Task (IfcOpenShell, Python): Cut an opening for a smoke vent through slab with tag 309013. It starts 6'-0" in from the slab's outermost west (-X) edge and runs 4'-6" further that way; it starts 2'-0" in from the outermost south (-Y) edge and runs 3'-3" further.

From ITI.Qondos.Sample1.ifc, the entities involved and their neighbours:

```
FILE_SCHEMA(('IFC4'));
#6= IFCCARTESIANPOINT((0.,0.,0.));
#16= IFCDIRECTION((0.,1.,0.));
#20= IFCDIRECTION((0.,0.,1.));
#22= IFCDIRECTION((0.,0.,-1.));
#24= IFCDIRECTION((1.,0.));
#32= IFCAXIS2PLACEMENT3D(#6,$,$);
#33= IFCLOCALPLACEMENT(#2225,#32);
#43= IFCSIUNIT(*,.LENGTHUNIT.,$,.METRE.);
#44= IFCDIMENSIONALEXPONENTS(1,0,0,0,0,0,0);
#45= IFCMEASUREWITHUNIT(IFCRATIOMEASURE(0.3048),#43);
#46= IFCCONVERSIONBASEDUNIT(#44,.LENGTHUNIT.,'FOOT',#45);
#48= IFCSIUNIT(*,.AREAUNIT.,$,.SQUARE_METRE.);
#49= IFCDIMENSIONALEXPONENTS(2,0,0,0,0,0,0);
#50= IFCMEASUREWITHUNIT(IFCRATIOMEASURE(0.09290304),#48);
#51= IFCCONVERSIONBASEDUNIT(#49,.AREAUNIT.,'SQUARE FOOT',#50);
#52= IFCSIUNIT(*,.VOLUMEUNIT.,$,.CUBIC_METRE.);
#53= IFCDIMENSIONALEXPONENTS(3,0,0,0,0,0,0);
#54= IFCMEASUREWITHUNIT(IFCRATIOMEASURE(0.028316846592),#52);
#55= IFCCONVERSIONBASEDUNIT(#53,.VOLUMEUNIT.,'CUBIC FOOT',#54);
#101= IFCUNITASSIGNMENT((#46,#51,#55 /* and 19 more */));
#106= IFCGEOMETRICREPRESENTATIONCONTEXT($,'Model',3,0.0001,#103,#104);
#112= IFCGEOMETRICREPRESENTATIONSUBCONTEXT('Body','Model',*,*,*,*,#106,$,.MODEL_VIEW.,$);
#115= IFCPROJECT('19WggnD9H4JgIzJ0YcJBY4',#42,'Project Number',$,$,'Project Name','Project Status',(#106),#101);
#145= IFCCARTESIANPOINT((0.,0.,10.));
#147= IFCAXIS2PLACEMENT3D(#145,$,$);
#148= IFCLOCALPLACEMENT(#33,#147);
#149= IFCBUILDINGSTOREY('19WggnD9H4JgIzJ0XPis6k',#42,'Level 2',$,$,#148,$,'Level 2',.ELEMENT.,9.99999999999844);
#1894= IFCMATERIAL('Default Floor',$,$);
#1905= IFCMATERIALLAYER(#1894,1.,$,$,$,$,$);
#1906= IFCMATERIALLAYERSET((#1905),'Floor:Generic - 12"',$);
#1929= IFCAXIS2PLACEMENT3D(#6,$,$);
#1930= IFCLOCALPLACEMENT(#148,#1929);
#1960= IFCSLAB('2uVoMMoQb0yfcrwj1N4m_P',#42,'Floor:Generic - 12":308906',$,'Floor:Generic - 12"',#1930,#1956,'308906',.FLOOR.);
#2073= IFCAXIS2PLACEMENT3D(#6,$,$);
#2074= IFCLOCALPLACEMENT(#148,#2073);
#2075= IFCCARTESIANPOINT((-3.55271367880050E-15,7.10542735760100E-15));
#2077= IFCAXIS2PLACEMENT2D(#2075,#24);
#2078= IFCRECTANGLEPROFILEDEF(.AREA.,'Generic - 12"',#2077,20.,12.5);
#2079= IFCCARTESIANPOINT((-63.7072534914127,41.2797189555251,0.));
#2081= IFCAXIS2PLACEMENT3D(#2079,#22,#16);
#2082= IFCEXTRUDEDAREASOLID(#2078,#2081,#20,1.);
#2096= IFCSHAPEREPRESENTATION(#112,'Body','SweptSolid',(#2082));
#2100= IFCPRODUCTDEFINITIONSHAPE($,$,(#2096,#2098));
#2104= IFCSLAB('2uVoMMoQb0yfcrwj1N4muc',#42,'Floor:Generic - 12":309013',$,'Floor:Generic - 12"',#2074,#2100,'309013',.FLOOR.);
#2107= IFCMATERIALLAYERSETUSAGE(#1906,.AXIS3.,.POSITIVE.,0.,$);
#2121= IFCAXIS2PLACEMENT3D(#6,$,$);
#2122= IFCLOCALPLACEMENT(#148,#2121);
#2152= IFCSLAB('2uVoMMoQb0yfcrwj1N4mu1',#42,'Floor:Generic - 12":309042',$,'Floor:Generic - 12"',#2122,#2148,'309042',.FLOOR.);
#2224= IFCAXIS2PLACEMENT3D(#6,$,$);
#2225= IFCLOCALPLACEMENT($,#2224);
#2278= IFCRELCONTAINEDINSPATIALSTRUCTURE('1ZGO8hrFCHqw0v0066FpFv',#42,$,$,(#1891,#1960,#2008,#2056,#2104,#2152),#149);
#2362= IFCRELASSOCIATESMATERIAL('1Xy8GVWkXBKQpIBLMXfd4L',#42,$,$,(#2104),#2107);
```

```python
import numpy as np
import ifcopenshell
import ifcopenshell.api.feature
import ifcopenshell.api.geometry
import ifcopenshell.api.root
import ifcopenshell.geom
import ifcopenshell.util.placement
import ifcopenshell.util.representation
import ifcopenshell.util.shape
import ifcopenshell.util.unit

model = ifcopenshell.open("ITI.Qondos.Sample1.ifc")
unit_scale = ifcopenshell.util.unit.calculate_unit_scale(model)
settings = ifcopenshell.geom.settings()


def volume(element):
    """Net volume in cubic metres, openings subtracted."""
    shape = ifcopenshell.geom.create_shape(settings, element)
    return ifcopenshell.util.shape.get_volume(shape.geometry)


slab = model.by_guid("2uVoMMoQb0yfcrwj1N4muc")
before = volume(slab)

# Extent in the slab's own axes, in metres. The edges named are its -X and -Y sides.
slab_shape = ifcopenshell.geom.create_shape(settings, slab)
vertices = ifcopenshell.util.shape.get_vertices(slab_shape.geometry)
x_min, y_min, bottom = vertices.min(axis=0)
top = vertices[:, 2].max()

opening = ifcopenshell.api.root.create_entity(model, ifc_class="IfcOpeningElement", name="Smoke vent opening", predefined_type="OPENING")
context = ifcopenshell.util.representation.get_context(model, "Model", "Body", "MODEL_VIEW")
width, depth = 1.3716, 0.9906
outline = [(0.0, 0.0), (width, 0.0), (width, depth), (0.0, depth), (0.0, 0.0)]
# Overshoot both faces by 50 mm so the cut is clean.
shape = ifcopenshell.api.geometry.add_slab_representation(
    model, context=context, depth=top - bottom + 0.1, polyline=outline
)
ifcopenshell.api.geometry.assign_representation(model, product=opening, representation=shape)

matrix = ifcopenshell.util.placement.get_local_placement(slab.ObjectPlacement)
matrix[:, 3] = matrix @ np.append(np.array([x_min + 1.8288, y_min + 0.6096, bottom - 0.05]) / unit_scale, 1.0)
ifcopenshell.api.geometry.edit_object_placement(model, product=opening, matrix=matrix, is_si=False)
ifcopenshell.api.feature.add_feature(model, feature=opening, element=slab)

after = volume(slab)

print(f"slab volume {before:.3f} -> {after:.3f} m3")

model.write("ITI.Qondos.Sample1_rev.ifc")
```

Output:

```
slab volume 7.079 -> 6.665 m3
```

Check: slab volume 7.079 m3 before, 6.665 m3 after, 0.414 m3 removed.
